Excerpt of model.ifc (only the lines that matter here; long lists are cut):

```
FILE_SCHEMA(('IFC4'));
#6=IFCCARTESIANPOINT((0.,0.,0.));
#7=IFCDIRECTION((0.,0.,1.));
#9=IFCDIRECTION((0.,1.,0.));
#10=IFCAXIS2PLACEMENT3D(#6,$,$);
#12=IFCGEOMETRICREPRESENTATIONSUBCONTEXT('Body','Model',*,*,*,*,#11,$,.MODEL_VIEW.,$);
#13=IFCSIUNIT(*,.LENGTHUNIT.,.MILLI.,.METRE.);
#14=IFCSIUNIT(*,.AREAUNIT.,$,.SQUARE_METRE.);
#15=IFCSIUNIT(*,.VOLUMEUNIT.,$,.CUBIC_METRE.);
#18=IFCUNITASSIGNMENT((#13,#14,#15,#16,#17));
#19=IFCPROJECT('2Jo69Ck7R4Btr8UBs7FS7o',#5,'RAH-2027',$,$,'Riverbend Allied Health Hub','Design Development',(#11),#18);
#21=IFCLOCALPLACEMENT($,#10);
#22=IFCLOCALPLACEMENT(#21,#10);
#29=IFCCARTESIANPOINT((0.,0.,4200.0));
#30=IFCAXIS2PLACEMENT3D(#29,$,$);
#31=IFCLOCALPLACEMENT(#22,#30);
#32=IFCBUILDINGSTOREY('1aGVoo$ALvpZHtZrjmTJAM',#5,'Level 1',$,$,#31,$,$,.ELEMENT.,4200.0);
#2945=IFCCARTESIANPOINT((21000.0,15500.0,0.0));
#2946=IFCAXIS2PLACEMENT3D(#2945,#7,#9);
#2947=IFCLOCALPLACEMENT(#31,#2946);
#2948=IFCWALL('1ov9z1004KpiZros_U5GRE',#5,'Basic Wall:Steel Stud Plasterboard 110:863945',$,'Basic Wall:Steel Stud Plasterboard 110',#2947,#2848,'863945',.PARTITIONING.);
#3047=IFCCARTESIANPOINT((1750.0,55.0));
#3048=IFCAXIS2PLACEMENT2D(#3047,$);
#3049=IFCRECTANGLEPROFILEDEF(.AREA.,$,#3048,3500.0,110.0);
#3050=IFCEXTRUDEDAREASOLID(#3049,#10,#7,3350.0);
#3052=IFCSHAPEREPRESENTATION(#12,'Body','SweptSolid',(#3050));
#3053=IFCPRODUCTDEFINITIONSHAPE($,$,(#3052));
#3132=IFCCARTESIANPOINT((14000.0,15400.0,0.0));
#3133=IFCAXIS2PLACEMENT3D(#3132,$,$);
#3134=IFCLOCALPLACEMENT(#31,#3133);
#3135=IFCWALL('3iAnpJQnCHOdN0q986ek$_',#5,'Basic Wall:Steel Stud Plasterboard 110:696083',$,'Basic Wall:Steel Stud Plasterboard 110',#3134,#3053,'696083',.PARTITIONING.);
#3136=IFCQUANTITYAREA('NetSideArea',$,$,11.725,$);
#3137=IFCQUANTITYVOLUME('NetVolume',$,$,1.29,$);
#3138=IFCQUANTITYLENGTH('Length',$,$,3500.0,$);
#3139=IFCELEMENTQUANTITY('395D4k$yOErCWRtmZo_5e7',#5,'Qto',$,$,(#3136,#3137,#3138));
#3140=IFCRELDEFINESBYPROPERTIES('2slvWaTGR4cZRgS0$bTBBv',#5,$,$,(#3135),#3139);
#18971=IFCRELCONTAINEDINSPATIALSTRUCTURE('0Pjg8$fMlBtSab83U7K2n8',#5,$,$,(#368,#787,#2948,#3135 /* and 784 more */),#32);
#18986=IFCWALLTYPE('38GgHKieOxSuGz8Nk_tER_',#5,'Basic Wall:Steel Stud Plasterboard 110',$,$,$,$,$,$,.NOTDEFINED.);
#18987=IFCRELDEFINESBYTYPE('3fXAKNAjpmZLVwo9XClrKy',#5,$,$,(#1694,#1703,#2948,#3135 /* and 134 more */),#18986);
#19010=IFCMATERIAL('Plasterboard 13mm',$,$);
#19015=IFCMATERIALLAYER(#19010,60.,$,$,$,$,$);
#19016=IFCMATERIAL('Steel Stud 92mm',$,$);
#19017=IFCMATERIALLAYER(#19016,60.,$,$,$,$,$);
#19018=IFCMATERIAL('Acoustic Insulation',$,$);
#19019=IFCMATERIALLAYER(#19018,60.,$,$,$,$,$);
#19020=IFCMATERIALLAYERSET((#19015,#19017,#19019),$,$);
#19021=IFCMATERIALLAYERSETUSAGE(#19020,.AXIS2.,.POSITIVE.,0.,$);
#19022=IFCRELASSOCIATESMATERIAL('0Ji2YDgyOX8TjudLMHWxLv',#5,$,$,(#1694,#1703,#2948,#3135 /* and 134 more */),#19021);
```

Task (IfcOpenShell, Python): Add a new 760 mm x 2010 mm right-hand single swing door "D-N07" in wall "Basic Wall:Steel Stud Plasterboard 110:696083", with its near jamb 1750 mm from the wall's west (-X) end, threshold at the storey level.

```python
import numpy as np
import ifcopenshell
import ifcopenshell.api.feature
import ifcopenshell.api.geometry
import ifcopenshell.api.pset
import ifcopenshell.api.root
import ifcopenshell.api.spatial
import ifcopenshell.geom
import ifcopenshell.util.element
import ifcopenshell.util.placement
import ifcopenshell.util.representation
import ifcopenshell.util.shape
import ifcopenshell.util.unit

model = ifcopenshell.open("model.ifc")
unit_scale = ifcopenshell.util.unit.calculate_unit_scale(model)
area_scale = ifcopenshell.util.unit.calculate_unit_scale(model, "AREAUNIT")
volume_scale = ifcopenshell.util.unit.calculate_unit_scale(model, "VOLUMEUNIT")
settings = ifcopenshell.geom.settings()


def volume(element):
    """Net volume in cubic metres, openings subtracted."""
    shape = ifcopenshell.geom.create_shape(settings, element)
    return ifcopenshell.util.shape.get_volume(shape.geometry)


wall = model.by_guid("3iAnpJQnCHOdN0q986ek$_")
storey = ifcopenshell.util.element.get_container(wall, ifc_class="IfcBuildingStorey")
context = ifcopenshell.util.representation.get_context(model, "Model", "Body", "MODEL_VIEW")
before = volume(wall)

width, height, from_end, sill = 0.76, 2.01, 1.75, 0.0  # metres

# The wall runs along its own X axis, and the end named is its -X end.
wall_shape = ifcopenshell.geom.create_shape(settings, wall)
x, y, z = ifcopenshell.util.shape.get_vertices(wall_shape.geometry).T
start = x.min() + from_end
face, thickness = float(y.min()), float(y.max() - y.min())
wall_matrix = ifcopenshell.util.placement.get_local_placement(wall.ObjectPlacement)
level = ifcopenshell.util.placement.get_local_placement(storey.ObjectPlacement)[2, 3]


def in_wall(x, y):
    """Placement at x, y metres in the wall's axes, at sill height."""
    matrix = wall_matrix.copy()
    matrix[:, 3] = wall_matrix @ np.array([x / unit_scale, y / unit_scale, 0.0, 1.0])
    matrix[2, 3] = level + sill / unit_scale
    return matrix


# Opening: a box that overshoots both wall faces by 50 mm.
opening = ifcopenshell.api.root.create_entity(model, ifc_class="IfcOpeningElement", predefined_type="OPENING")
box = ifcopenshell.api.geometry.add_wall_representation(
    model, context=context, length=width, height=height, thickness=thickness + 0.1
)
ifcopenshell.api.geometry.assign_representation(model, product=opening, representation=box)
ifcopenshell.api.geometry.edit_object_placement(model, product=opening, matrix=in_wall(start, face - 0.05), is_si=False)
ifcopenshell.api.feature.add_feature(model, feature=opening, element=wall)

door = ifcopenshell.api.root.create_entity(model, ifc_class="IfcDoor", name="D-N07", predefined_type="DOOR")
door.OverallWidth, door.OverallHeight = width / unit_scale, height / unit_scale
door.OperationType = "SINGLE_SWING_RIGHT"
body = ifcopenshell.api.geometry.add_door_representation(
    model,
    context=context,
    overall_width=door.OverallWidth,
    overall_height=door.OverallHeight,
    operation_type="SINGLE_SWING_RIGHT",
    lining_properties={"LiningDepth": thickness / unit_scale, "ThresholdDepth": thickness / unit_scale},
)
ifcopenshell.api.geometry.assign_representation(model, product=door, representation=body)
ifcopenshell.api.spatial.assign_container(model, products=[door], relating_structure=storey)
ifcopenshell.api.feature.add_filling(model, opening=opening, element=door)

# The lining spans the wall, so the door starts at the wall face.
ifcopenshell.api.geometry.edit_object_placement(model, product=door, matrix=in_wall(start, face), is_si=False)

after = volume(wall)

# Update the wall's stored quantities.
qto = model.by_id(ifcopenshell.util.element.get_pset(wall, "Qto", should_inherit=False)["id"])
ifcopenshell.api.pset.edit_qto(model, qto=qto, properties={
    "NetSideArea": after / thickness / area_scale,
    "NetVolume": after / volume_scale,
})

print(f"wall volume {before:.3f} -> {after:.3f} m3")

model.write("model_v2.ifc")
```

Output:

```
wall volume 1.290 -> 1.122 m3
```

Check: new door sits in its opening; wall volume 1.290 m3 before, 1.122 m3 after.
